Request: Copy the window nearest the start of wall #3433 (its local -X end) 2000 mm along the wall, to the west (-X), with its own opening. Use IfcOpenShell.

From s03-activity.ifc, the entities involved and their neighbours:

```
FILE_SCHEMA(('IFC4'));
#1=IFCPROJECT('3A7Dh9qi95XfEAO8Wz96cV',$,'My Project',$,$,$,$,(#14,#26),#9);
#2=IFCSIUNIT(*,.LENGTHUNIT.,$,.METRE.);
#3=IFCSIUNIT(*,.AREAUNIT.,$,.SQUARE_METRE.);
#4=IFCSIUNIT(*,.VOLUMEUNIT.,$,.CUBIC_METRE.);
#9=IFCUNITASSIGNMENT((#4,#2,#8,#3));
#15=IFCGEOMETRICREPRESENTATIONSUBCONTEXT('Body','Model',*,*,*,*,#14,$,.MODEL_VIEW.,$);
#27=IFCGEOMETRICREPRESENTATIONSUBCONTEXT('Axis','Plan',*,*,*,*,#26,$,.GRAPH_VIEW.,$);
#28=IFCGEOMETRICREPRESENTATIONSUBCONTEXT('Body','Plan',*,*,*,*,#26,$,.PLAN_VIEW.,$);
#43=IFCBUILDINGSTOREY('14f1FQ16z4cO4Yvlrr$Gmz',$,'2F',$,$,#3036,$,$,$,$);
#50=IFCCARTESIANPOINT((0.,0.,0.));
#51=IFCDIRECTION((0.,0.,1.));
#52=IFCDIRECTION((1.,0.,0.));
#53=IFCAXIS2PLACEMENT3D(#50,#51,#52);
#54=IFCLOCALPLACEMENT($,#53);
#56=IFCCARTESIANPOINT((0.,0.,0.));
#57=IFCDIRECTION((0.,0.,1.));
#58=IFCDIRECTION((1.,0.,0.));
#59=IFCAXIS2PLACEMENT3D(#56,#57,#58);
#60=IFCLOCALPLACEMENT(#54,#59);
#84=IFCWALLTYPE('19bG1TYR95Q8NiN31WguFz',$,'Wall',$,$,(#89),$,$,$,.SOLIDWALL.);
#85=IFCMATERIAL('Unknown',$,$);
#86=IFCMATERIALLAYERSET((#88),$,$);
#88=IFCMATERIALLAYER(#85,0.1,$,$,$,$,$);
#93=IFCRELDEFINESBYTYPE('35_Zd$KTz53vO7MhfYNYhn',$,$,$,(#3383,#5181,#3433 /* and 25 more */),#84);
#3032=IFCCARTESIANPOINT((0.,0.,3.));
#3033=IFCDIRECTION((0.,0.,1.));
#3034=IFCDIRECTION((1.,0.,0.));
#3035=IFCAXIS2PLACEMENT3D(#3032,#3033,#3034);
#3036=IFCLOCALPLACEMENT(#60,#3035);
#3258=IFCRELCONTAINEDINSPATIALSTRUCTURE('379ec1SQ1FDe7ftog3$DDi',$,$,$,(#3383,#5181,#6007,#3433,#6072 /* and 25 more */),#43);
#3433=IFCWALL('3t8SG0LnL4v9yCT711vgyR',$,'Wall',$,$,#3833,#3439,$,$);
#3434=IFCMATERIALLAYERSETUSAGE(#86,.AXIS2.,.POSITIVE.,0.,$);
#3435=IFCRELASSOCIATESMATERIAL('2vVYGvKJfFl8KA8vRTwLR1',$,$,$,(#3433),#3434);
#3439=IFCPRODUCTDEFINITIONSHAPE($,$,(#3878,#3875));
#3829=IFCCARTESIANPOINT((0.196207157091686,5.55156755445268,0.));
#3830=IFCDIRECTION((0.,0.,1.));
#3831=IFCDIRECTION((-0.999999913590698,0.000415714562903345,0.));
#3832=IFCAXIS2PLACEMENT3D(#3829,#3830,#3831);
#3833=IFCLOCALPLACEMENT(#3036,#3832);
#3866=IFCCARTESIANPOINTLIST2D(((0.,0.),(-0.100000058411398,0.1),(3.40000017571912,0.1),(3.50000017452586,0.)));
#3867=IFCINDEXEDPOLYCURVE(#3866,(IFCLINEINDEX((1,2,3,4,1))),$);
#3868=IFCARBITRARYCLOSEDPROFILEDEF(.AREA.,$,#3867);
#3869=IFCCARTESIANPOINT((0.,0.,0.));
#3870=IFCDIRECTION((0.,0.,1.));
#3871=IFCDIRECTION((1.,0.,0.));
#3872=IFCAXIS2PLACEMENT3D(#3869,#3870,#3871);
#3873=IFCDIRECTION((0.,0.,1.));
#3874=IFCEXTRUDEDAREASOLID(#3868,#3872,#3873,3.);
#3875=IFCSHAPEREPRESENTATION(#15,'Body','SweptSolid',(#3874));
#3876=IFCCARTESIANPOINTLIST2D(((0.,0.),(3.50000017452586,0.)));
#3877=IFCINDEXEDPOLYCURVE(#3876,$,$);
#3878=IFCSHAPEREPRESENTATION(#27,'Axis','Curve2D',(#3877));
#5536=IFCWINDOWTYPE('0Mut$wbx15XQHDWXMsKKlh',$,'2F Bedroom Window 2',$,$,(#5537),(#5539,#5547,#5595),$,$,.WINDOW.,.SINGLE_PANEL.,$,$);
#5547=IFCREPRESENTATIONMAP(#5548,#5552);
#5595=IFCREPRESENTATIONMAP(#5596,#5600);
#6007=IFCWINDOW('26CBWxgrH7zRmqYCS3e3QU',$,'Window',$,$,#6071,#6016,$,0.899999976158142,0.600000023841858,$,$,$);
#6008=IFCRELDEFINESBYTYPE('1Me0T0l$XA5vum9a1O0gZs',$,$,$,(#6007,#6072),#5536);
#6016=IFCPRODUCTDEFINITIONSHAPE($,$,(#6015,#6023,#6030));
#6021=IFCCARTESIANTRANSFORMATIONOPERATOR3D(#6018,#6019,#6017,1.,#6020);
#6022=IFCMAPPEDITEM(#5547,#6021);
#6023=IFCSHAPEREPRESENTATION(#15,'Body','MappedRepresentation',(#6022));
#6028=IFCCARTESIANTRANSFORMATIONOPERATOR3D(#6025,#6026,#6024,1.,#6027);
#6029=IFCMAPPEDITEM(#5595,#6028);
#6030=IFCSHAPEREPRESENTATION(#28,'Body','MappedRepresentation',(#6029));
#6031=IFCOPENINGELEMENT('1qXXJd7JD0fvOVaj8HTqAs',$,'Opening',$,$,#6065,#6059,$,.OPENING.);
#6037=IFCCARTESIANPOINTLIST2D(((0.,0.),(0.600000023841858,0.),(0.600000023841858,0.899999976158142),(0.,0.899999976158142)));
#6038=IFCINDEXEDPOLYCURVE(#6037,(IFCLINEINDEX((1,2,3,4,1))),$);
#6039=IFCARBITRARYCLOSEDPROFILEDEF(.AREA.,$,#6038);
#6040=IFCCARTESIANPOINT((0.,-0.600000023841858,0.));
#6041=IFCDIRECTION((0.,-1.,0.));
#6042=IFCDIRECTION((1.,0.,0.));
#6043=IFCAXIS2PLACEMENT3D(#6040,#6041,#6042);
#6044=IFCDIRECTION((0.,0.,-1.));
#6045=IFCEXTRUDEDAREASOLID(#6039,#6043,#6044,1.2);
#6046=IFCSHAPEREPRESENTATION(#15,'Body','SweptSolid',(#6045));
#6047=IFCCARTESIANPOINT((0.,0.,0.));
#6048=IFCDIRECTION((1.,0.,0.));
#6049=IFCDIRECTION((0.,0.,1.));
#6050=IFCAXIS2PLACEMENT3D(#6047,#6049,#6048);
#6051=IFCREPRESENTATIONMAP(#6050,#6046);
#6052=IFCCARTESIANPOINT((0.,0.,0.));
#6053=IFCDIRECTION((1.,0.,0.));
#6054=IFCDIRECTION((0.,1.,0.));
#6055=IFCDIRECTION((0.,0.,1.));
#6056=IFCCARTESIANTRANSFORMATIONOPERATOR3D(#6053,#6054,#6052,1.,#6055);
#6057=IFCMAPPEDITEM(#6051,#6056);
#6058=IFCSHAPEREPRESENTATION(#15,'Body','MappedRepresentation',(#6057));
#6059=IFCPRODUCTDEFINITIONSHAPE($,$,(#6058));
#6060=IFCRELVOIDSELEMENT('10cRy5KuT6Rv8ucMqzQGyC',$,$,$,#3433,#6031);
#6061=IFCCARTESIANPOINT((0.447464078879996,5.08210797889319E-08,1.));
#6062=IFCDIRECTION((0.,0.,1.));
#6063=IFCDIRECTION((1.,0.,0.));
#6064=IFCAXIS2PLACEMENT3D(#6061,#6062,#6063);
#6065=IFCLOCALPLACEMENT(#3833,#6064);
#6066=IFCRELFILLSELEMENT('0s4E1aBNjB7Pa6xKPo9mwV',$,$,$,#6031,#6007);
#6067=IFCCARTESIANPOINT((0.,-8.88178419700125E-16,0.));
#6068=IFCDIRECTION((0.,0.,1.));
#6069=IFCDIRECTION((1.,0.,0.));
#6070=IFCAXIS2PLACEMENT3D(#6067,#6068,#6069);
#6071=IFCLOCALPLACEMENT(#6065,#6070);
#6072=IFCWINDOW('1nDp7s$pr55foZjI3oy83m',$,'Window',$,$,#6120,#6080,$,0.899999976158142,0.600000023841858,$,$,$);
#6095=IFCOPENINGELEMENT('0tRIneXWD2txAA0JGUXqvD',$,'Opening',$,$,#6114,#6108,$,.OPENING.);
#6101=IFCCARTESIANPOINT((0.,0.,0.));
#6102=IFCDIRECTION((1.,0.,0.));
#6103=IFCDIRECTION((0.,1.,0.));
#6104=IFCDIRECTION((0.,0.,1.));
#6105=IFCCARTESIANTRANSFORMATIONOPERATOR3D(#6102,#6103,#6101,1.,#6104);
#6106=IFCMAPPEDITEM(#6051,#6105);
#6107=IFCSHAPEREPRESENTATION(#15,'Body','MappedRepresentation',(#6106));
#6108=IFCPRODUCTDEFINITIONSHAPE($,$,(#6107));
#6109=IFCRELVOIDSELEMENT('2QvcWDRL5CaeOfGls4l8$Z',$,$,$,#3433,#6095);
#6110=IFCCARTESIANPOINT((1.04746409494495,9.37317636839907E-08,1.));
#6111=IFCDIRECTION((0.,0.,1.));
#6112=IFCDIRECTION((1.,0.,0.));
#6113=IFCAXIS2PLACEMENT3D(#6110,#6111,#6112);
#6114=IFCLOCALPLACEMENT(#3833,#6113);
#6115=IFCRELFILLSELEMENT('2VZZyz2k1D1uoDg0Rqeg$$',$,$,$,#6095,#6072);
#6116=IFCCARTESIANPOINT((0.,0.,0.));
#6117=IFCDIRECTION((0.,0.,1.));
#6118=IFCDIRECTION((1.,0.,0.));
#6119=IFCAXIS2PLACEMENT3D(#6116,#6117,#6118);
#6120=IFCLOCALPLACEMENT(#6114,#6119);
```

```python
import ifcopenshell
import ifcopenshell.api.feature
import ifcopenshell.api.geometry
import ifcopenshell.api.root
import ifcopenshell.geom
import ifcopenshell.util.element
import ifcopenshell.util.placement
import ifcopenshell.util.shape
import ifcopenshell.util.unit

model = ifcopenshell.open("s03-activity.ifc")
unit_scale = ifcopenshell.util.unit.calculate_unit_scale(model)
settings = ifcopenshell.geom.settings()


def volume(element):
    """Net volume in cubic metres, openings subtracted."""
    shape = ifcopenshell.geom.create_shape(settings, element)
    return ifcopenshell.util.shape.get_volume(shape.geometry)


window = model.by_guid("26CBWxgrH7zRmqYCS3e3QU")
opening = window.FillsVoids[0].RelatingOpeningElement
wall = opening.VoidsElements[0].RelatingBuildingElement
before = volume(wall)
shift = ifcopenshell.util.placement.get_local_placement(wall.ObjectPlacement)[:3, 0] * 2 / unit_scale

# copy_class copies the void relationship, type, container and properties, but no geometry.
new_opening = ifcopenshell.api.root.copy_class(model, product=opening)
new_opening.Representation = ifcopenshell.util.element.copy_deep(
    model, opening.Representation, exclude=["IfcGeometricRepresentationContext", "IfcRepresentationMap"]
)
new_window = ifcopenshell.api.root.copy_class(model, product=window)
new_window.Representation = ifcopenshell.util.element.copy_deep(
    model, window.Representation, exclude=["IfcGeometricRepresentationContext", "IfcRepresentationMap"]
)
ifcopenshell.api.feature.add_filling(model, opening=new_opening, element=new_window)

for old, new in ((opening, new_opening), (window, new_window)):
    matrix = ifcopenshell.util.placement.get_local_placement(old.ObjectPlacement)
    matrix[:3, 3] += shift
    ifcopenshell.api.geometry.edit_object_placement(model, product=new, matrix=matrix, is_si=False)

after = volume(wall)

print(f"wall volume {before:.3f} -> {after:.3f} m3")

model.write("s03-activity_edited.ifc")
```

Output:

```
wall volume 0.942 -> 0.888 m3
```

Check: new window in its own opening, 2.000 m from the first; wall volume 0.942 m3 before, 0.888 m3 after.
